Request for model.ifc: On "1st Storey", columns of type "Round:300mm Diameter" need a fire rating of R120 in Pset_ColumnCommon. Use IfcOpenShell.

First a look at what the model holds.

```python
import ifcopenshell
import ifcopenshell.util.element

model = ifcopenshell.open("model.ifc")
print(model.schema)
storey = next(s for s in model.by_type("IfcBuildingStorey") if s.Name == "1st Storey")
columns = [e for e in ifcopenshell.util.element.get_decomposition(storey) if e.is_a("IfcColumn")]
seen = {}
for e in columns:
    element_type = ifcopenshell.util.element.get_type(e)
    key = (element_type.Name if element_type != e and element_type else None, ifcopenshell.util.element.get_pset(e, "Pset_ColumnCommon", "FireRating"))
    seen[key] = seen.get(key, 0) + 1
for (name, value), count in sorted(seen.items(), key=str):
    print(count, "x", name, "|", value)
```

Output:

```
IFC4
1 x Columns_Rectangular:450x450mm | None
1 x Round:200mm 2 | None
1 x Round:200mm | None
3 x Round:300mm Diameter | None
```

```python
import ifcopenshell
import ifcopenshell.api.pset
import ifcopenshell.util.element

model = ifcopenshell.open("model.ifc")

storey = next(s for s in model.by_type("IfcBuildingStorey") if s.Name == "1st Storey")
columns = [e for e in ifcopenshell.util.element.get_decomposition(storey) if e.is_a("IfcColumn")]

count = 0
for e in columns:
    element_type = ifcopenshell.util.element.get_type(e)
    if element_type in (None, e) or element_type.Name != "Round:300mm Diameter":
        continue
    # add_pset returns the element's existing set when there is one.
    pset = ifcopenshell.api.pset.add_pset(model, product=e, name="Pset_ColumnCommon")
    ifcopenshell.api.pset.edit_pset(model, pset=pset, properties={"FireRating": "R120"})
    count += 1

print(count, "columns updated")

model.write("model_v2.ifc")
```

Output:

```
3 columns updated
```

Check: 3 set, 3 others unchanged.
